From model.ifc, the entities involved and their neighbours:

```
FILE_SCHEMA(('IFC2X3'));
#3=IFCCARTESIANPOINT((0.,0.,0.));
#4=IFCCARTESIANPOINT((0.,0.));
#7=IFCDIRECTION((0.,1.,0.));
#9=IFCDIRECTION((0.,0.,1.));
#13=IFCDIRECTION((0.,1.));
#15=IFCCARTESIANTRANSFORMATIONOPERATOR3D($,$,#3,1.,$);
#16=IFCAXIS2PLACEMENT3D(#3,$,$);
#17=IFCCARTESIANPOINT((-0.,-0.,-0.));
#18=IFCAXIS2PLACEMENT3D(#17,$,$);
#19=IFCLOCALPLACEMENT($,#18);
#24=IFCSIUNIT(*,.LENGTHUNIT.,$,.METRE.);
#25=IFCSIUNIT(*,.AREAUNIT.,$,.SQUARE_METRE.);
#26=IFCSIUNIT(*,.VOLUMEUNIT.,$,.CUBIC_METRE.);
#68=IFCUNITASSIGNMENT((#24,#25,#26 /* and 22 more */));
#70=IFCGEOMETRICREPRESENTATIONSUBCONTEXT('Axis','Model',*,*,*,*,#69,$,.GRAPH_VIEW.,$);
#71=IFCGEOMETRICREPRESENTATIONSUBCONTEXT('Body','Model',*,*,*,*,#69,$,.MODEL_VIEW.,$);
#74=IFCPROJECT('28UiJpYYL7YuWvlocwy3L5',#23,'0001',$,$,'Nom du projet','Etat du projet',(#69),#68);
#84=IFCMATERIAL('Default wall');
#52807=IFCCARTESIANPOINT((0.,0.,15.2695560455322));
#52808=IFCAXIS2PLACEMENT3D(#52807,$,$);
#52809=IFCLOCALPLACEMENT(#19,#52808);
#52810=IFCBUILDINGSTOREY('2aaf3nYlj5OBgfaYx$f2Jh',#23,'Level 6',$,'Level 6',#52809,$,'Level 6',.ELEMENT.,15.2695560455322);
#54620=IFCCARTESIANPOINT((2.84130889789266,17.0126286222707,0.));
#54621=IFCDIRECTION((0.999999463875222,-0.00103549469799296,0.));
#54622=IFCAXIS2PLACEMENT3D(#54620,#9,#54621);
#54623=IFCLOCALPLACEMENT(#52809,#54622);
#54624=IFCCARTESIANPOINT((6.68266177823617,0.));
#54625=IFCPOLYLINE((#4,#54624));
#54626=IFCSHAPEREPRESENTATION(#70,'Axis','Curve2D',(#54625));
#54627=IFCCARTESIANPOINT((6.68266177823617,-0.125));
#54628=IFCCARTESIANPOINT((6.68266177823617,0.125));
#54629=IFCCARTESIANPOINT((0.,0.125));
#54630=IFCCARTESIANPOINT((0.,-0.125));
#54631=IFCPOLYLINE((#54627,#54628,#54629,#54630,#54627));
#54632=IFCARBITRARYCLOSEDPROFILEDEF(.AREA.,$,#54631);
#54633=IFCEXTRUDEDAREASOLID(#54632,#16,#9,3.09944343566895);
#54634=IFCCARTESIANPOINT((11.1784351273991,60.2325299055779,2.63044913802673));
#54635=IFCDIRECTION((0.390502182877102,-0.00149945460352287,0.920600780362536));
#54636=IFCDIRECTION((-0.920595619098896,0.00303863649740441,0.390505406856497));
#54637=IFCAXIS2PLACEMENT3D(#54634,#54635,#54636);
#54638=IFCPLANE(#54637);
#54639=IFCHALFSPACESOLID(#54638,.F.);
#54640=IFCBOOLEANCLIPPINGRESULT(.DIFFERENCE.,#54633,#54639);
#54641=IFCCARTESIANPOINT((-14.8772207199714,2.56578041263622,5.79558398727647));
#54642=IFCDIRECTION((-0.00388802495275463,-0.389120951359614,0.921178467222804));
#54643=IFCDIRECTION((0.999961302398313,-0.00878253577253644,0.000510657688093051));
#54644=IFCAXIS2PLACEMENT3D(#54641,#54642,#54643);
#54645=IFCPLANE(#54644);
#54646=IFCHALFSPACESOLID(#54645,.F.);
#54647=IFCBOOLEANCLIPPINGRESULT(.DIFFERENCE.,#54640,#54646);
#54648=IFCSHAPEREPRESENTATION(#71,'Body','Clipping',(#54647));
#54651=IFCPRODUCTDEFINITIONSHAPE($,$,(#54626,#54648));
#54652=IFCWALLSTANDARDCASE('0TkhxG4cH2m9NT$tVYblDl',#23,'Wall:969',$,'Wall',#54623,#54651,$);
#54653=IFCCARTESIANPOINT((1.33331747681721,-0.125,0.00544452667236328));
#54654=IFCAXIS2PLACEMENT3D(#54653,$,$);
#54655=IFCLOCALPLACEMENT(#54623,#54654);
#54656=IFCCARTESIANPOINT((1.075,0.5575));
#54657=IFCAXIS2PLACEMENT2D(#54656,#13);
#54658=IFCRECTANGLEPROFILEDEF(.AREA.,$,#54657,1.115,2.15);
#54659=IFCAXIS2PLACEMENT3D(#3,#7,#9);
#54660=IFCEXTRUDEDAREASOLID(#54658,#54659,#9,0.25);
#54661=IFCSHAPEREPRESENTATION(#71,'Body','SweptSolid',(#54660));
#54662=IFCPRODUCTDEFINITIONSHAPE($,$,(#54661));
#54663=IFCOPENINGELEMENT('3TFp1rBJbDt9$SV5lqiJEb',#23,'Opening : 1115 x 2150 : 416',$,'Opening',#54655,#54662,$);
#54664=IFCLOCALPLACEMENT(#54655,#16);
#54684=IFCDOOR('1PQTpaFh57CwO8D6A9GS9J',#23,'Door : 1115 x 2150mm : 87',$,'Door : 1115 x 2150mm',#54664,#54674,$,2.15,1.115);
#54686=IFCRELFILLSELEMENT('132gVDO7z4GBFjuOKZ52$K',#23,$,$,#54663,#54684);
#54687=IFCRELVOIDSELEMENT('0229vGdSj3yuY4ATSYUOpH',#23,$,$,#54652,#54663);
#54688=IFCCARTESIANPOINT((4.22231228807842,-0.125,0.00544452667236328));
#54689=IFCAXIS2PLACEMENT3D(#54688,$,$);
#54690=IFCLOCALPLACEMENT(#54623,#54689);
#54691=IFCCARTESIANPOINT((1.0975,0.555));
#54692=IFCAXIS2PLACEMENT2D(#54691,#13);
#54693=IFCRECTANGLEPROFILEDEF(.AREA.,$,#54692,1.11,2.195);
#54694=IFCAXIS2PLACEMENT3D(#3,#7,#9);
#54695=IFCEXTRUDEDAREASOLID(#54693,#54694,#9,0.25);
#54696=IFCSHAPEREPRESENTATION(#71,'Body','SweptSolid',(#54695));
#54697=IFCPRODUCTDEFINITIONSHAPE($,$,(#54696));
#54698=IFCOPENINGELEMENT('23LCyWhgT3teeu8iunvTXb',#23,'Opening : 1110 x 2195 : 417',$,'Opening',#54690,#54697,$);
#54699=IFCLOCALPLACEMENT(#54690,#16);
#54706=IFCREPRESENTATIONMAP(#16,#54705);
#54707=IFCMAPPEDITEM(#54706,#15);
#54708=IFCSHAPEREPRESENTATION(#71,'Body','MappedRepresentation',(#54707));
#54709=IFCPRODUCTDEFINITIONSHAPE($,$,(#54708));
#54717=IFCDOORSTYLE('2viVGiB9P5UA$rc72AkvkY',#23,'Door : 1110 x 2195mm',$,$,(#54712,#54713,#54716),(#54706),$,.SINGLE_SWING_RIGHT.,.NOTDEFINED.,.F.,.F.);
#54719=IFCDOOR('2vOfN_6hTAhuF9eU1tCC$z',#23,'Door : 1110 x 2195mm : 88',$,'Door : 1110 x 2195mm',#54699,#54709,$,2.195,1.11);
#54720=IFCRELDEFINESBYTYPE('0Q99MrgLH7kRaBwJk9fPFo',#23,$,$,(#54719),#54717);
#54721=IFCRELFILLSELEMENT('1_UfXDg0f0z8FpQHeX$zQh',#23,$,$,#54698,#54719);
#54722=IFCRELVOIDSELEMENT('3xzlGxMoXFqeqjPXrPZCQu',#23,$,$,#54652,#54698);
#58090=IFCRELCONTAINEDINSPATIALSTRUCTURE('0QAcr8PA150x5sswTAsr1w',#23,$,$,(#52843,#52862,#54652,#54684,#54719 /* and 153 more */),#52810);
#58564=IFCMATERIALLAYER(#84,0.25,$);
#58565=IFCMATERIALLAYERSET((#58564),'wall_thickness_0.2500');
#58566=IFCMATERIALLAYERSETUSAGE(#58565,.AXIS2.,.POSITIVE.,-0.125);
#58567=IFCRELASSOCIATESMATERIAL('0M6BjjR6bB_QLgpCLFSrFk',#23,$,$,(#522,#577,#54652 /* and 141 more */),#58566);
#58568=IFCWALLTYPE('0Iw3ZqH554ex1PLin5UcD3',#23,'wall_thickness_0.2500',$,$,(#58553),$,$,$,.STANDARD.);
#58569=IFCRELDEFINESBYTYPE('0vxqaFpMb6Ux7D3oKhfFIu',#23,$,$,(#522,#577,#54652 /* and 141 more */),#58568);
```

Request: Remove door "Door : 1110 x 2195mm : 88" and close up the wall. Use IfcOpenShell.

```python
import ifcopenshell
import ifcopenshell.api.feature
import ifcopenshell.api.root
import ifcopenshell.geom
import ifcopenshell.util.shape

model = ifcopenshell.open("model.ifc")
settings = ifcopenshell.geom.settings()


def volume(element):
    """Net volume in cubic metres, openings subtracted."""
    shape = ifcopenshell.geom.create_shape(settings, element)
    return ifcopenshell.util.shape.get_volume(shape.geometry)


door = model.by_guid("2vOfN_6hTAhuF9eU1tCC$z")
opening = door.FillsVoids[0].RelatingOpeningElement
wall = opening.VoidsElements[0].RelatingBuildingElement
before = volume(wall)

ifcopenshell.api.root.remove_product(model, product=door)
ifcopenshell.api.feature.remove_feature(model, feature=opening)

after = volume(wall)

print(f"wall volume {before:.3f} -> {after:.3f} m3")

model.write("model_rev.ifc")
```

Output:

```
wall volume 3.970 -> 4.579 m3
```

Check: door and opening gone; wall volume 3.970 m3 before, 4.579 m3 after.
